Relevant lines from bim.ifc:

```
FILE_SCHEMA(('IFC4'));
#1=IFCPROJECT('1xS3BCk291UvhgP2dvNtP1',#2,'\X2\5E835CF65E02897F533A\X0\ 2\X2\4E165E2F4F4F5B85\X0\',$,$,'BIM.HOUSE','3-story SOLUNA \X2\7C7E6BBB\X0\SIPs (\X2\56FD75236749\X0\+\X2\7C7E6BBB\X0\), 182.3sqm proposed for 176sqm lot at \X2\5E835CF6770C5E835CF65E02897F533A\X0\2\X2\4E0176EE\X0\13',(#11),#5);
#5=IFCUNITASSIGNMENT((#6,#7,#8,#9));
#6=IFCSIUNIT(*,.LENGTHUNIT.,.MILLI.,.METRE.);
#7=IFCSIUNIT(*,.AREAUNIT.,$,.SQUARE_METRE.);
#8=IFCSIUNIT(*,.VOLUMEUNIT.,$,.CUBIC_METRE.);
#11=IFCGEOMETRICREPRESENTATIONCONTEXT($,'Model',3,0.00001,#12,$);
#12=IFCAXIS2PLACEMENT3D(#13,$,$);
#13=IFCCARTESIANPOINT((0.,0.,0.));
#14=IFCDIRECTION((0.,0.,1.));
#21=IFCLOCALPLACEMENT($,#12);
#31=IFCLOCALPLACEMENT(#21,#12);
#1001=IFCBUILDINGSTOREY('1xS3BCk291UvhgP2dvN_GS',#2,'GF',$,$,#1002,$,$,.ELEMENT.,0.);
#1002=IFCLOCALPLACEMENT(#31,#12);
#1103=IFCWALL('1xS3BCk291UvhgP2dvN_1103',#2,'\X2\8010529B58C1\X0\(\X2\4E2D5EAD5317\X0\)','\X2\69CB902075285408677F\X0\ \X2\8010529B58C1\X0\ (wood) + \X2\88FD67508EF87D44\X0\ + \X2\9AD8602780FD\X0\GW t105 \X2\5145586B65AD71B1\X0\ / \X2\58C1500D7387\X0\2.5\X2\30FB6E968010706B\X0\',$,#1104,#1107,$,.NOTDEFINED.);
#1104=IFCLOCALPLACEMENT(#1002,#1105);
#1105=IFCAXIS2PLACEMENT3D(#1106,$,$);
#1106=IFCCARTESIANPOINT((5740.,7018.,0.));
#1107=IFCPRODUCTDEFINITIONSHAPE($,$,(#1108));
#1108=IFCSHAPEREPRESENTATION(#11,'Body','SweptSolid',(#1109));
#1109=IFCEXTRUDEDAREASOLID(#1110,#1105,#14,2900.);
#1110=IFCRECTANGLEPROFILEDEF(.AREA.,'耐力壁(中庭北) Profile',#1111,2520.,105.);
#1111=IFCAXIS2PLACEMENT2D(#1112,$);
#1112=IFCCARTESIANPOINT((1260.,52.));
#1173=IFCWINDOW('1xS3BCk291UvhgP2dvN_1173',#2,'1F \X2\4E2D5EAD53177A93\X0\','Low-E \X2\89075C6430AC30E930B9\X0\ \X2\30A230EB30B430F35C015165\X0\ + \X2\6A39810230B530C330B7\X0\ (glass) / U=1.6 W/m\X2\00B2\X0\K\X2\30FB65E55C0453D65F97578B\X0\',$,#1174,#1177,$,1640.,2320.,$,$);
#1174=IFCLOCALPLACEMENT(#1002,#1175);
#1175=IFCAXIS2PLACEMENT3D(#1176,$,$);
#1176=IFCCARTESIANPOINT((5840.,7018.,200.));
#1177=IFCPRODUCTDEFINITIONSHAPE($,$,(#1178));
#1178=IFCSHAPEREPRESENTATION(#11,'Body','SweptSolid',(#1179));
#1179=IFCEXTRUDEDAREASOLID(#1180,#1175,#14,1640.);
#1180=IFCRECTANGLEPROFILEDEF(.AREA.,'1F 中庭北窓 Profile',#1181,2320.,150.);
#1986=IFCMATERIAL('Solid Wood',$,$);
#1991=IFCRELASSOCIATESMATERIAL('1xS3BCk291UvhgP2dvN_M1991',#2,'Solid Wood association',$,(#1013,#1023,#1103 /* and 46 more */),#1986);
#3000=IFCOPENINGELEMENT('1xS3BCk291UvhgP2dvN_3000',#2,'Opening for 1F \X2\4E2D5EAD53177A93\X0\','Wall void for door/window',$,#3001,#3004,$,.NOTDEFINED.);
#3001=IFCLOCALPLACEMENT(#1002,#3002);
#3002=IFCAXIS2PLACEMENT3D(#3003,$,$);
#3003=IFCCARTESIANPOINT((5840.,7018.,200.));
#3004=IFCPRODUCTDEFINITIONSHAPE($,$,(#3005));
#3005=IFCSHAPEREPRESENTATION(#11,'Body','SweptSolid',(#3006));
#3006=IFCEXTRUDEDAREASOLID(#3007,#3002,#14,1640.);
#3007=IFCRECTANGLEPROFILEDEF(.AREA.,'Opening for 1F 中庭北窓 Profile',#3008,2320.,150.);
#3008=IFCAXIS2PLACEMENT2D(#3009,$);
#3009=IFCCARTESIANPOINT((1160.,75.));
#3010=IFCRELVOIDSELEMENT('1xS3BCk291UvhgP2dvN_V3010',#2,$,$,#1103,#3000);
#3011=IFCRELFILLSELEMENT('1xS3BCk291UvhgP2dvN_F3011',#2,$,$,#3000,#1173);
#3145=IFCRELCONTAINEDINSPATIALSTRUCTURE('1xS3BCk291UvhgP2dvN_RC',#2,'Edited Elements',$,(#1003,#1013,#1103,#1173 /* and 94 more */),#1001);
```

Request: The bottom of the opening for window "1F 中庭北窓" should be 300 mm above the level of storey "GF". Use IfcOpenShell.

```python
import numpy as np
import ifcopenshell
import ifcopenshell.api.geometry
import ifcopenshell.geom
import ifcopenshell.util.element
import ifcopenshell.util.placement
import ifcopenshell.util.shape
import ifcopenshell.util.unit

model = ifcopenshell.open("bim.ifc")
unit_scale = ifcopenshell.util.unit.calculate_unit_scale(model)

window = model.by_guid("1xS3BCk291UvhgP2dvN_1173")
opening = window.FillsVoids[0].RelatingOpeningElement
storey = ifcopenshell.util.element.get_container(window, ifc_class="IfcBuildingStorey")
level = ifcopenshell.util.placement.get_local_placement(storey.ObjectPlacement)[2, 3]

# The opening's origin need not be at the sill, so measure its lowest point.
shape = ifcopenshell.geom.create_shape(ifcopenshell.geom.settings(), opening)
bottom = ifcopenshell.util.shape.get_shape_bottom_elevation(shape, shape.geometry) / unit_scale
dz = level + 0.3 / unit_scale - bottom

shift = np.array([0.0, 0.0, dz])
# The window is not placed relative to its opening, so move both.
for product in (opening, window):
    matrix = ifcopenshell.util.placement.get_local_placement(product.ObjectPlacement)
    matrix[:3, 3] += shift
    ifcopenshell.api.geometry.edit_object_placement(model, product=product, matrix=matrix, is_si=False)

print(f"moved by {dz * unit_scale:+.3f} m")

model.write("bim-out.ifc")
```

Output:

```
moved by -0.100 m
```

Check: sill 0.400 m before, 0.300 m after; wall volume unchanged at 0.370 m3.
